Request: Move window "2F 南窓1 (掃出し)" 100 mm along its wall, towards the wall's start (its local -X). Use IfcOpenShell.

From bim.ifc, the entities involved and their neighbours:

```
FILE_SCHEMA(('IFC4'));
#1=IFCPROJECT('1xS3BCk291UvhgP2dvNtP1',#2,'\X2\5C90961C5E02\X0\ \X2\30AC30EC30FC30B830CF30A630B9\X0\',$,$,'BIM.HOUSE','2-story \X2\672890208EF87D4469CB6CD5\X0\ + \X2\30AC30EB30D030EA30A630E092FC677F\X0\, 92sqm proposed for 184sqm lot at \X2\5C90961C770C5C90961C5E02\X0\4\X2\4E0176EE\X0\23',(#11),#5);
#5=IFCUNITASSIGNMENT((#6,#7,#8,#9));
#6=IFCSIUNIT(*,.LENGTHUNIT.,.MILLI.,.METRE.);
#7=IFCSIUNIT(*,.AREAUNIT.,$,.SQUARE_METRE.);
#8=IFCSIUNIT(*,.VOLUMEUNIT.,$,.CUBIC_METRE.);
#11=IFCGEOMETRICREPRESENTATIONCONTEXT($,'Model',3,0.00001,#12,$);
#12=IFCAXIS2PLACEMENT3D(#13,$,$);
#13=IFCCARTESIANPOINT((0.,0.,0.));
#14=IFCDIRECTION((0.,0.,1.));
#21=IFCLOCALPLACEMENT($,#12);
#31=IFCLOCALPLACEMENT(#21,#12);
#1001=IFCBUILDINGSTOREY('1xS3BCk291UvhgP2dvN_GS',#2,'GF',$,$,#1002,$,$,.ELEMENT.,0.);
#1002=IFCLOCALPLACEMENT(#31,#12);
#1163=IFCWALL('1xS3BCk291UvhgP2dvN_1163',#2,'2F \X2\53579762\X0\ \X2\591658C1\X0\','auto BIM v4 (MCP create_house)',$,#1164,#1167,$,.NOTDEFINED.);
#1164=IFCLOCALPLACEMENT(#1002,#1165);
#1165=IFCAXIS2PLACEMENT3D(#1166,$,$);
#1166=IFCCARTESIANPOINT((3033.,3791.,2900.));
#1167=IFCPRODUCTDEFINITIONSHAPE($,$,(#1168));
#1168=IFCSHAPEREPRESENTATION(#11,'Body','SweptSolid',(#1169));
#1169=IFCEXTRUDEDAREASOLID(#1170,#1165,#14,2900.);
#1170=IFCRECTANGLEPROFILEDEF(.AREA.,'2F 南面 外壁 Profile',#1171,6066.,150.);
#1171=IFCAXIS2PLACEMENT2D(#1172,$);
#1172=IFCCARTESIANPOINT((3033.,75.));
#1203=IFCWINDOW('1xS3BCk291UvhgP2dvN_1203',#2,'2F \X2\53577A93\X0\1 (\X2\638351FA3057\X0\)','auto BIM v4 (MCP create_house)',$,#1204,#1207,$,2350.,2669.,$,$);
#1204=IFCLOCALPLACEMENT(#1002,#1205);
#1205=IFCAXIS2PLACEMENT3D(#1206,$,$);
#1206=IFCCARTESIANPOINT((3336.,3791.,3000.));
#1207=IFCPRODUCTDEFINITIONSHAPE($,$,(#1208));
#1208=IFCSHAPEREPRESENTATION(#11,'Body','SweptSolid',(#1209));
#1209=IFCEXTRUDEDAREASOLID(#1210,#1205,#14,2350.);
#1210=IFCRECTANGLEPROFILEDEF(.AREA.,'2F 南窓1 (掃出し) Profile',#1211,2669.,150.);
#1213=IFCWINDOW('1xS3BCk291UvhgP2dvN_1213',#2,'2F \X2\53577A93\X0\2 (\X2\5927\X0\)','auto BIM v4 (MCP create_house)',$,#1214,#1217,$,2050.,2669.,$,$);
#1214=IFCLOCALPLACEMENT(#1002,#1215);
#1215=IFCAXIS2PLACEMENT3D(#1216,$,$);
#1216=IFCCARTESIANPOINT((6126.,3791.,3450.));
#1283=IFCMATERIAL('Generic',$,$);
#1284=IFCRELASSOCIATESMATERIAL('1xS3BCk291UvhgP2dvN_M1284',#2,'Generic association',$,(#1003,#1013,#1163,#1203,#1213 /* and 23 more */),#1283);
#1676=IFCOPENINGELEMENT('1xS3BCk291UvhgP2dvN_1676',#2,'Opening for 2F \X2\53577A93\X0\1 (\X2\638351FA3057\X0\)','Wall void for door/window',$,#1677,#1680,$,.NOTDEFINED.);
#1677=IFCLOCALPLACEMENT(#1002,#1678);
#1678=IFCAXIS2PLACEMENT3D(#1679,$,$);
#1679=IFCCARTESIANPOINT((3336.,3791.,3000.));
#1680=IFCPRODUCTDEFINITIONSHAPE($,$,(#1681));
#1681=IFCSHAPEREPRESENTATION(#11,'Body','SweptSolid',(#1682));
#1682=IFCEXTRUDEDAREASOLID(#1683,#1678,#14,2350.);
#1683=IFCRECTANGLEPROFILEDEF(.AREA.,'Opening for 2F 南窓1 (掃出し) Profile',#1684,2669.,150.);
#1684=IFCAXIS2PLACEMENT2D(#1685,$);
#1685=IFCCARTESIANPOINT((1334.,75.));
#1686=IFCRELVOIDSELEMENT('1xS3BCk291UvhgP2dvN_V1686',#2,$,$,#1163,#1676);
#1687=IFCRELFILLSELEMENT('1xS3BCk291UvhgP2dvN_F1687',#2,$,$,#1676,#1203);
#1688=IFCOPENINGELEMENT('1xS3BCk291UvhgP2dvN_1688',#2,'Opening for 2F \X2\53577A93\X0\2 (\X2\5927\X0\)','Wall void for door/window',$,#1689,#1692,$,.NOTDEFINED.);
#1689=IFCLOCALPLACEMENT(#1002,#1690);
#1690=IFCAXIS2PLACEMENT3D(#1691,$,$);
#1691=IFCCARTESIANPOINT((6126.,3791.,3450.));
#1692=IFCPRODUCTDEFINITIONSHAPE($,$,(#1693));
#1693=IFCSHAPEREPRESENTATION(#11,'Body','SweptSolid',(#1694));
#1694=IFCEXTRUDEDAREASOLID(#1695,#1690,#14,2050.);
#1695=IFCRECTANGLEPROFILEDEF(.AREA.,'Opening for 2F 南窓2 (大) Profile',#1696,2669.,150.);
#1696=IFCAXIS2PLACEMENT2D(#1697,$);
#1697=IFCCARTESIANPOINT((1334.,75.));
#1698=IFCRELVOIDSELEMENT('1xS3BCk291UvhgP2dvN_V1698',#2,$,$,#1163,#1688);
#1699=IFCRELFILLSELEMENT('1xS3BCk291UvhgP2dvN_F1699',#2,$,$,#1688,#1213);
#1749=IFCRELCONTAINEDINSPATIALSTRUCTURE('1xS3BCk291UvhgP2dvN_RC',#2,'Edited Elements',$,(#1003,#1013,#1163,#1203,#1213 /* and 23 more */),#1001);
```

```python
import ifcopenshell
import ifcopenshell.api.geometry
import ifcopenshell.util.placement

model = ifcopenshell.open("bim.ifc")

window = model.by_guid("1xS3BCk291UvhgP2dvN_1203")
opening = window.FillsVoids[0].RelatingOpeningElement
wall = opening.VoidsElements[0].RelatingBuildingElement

wall_matrix = ifcopenshell.util.placement.get_local_placement(wall.ObjectPlacement)
shift = wall_matrix[:3, 0] * -100.0
before = ifcopenshell.util.placement.get_local_placement(window.ObjectPlacement)[:3, 3].copy()

# The window is not placed relative to its opening, so move both.
for product in (opening, window):
    matrix = ifcopenshell.util.placement.get_local_placement(product.ObjectPlacement)
    matrix[:3, 3] += shift
    ifcopenshell.api.geometry.edit_object_placement(model, product=product, matrix=matrix, is_si=False)

after = ifcopenshell.util.placement.get_local_placement(window.ObjectPlacement)[:3, 3]
print("window moved by", (after - before).round(3) + 0.0)

model.write("bim_updated.ifc")
```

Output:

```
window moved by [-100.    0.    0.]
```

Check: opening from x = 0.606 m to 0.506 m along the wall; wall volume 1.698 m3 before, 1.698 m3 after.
